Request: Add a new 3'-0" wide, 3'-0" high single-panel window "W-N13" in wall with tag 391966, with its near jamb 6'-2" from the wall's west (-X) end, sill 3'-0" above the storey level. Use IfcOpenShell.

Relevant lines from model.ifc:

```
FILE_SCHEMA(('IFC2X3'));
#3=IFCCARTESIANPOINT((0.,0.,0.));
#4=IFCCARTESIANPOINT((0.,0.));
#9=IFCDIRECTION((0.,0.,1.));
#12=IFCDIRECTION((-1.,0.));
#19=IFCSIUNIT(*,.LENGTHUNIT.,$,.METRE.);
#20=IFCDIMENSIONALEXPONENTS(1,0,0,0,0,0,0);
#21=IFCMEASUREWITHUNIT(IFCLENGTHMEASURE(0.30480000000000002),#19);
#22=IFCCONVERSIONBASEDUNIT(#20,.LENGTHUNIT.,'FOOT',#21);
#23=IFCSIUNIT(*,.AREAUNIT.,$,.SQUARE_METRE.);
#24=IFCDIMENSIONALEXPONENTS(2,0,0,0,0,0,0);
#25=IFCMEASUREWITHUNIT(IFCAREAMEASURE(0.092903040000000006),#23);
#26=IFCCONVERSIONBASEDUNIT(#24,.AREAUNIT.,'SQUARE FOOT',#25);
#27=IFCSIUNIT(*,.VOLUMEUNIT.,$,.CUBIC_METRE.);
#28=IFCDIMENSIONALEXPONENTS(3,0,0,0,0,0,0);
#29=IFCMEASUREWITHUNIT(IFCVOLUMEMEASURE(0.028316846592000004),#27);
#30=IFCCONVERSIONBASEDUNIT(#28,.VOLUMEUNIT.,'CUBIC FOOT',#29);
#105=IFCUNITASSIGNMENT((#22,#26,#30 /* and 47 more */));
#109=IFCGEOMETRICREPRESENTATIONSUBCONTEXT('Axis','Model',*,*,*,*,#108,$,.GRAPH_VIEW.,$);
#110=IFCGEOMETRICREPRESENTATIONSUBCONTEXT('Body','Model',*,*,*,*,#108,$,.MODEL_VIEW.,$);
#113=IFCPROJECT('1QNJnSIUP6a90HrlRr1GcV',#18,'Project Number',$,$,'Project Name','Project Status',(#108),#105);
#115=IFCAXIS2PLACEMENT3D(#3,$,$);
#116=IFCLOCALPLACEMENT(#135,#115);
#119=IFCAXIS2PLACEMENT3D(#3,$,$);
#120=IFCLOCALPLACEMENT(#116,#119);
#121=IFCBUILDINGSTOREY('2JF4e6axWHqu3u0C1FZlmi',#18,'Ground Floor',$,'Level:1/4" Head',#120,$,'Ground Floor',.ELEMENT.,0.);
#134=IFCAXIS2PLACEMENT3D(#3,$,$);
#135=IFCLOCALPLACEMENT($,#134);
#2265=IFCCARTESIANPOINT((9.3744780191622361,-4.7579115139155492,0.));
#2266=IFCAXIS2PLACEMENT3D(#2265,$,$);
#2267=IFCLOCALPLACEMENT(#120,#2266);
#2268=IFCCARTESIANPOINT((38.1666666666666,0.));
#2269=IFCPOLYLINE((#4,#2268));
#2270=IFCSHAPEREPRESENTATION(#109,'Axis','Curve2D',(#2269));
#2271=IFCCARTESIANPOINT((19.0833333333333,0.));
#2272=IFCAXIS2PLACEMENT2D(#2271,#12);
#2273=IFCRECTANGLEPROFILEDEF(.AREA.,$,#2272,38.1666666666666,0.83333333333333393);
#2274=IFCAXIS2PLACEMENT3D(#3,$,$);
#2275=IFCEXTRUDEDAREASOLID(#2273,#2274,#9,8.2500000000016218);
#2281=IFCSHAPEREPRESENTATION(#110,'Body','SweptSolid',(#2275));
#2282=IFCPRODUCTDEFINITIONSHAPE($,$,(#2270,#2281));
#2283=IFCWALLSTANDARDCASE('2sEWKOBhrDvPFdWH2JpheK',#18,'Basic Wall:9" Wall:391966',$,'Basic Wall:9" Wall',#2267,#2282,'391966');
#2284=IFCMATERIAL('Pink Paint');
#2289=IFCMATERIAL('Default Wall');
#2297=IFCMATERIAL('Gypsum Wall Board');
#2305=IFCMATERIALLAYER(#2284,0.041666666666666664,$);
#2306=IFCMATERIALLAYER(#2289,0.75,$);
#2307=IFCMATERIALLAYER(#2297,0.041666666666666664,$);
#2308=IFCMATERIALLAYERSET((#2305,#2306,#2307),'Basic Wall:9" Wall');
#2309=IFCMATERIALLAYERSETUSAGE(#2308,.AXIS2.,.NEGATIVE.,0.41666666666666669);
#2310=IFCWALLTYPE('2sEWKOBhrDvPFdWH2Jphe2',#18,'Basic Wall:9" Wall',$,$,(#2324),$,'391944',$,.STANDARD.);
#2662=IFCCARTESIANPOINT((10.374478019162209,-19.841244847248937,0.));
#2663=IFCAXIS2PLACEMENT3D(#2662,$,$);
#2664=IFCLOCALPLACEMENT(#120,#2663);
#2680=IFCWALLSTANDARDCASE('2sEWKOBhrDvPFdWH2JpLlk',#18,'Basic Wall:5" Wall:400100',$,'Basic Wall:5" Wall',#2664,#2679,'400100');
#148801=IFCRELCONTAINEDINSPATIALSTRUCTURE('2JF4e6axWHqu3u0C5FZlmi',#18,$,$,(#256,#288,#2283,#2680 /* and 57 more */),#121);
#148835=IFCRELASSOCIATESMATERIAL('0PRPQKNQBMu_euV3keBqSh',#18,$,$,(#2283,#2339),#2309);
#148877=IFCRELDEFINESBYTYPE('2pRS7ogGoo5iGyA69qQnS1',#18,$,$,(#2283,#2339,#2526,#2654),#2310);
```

```python
import numpy as np
import ifcopenshell
import ifcopenshell.api.feature
import ifcopenshell.api.geometry
import ifcopenshell.api.root
import ifcopenshell.api.spatial
import ifcopenshell.api.type
import ifcopenshell.geom
import ifcopenshell.util.element
import ifcopenshell.util.placement
import ifcopenshell.util.representation
import ifcopenshell.util.shape
import ifcopenshell.util.unit

model = ifcopenshell.open("model.ifc")
unit_scale = ifcopenshell.util.unit.calculate_unit_scale(model)
settings = ifcopenshell.geom.settings()


def volume(element):
    """Net volume in cubic metres, openings subtracted."""
    shape = ifcopenshell.geom.create_shape(settings, element)
    return ifcopenshell.util.shape.get_volume(shape.geometry)


wall = model.by_guid("2sEWKOBhrDvPFdWH2JpheK")
storey = ifcopenshell.util.element.get_container(wall, ifc_class="IfcBuildingStorey")
context = ifcopenshell.util.representation.get_context(model, "Model", "Body", "MODEL_VIEW")
before = volume(wall)

width, height, from_end, sill = 0.9144, 0.9144, 1.8796, 0.9144  # metres

# The wall runs along its own X axis, and the end named is its -X end.
wall_shape = ifcopenshell.geom.create_shape(settings, wall)
x, y, z = ifcopenshell.util.shape.get_vertices(wall_shape.geometry).T
start = x.min() + from_end
face, thickness = float(y.min()), float(y.max() - y.min())
wall_matrix = ifcopenshell.util.placement.get_local_placement(wall.ObjectPlacement)
level = ifcopenshell.util.placement.get_local_placement(storey.ObjectPlacement)[2, 3]


def in_wall(x, y):
    """Placement at x, y metres in the wall's axes, at sill height."""
    matrix = wall_matrix.copy()
    matrix[:, 3] = wall_matrix @ np.array([x / unit_scale, y / unit_scale, 0.0, 1.0])
    matrix[2, 3] = level + sill / unit_scale
    return matrix


# Opening: a box that overshoots both wall faces by 50 mm.
opening = ifcopenshell.api.root.create_entity(model, ifc_class="IfcOpeningElement")
box = ifcopenshell.api.geometry.add_wall_representation(
    model, context=context, length=width, height=height, thickness=thickness + 0.1
)
ifcopenshell.api.geometry.assign_representation(model, product=opening, representation=box)
ifcopenshell.api.geometry.edit_object_placement(model, product=opening, matrix=in_wall(start, face - 0.05), is_si=False)
ifcopenshell.api.feature.add_feature(model, feature=opening, element=wall)

window = ifcopenshell.api.root.create_entity(model, ifc_class="IfcWindow", name="W-N13")
window.OverallWidth, window.OverallHeight = width / unit_scale, height / unit_scale
body = ifcopenshell.api.geometry.add_window_representation(
    model,
    context=context,
    overall_width=window.OverallWidth,
    overall_height=window.OverallHeight,
    partition_type="SINGLE_PANEL",
)
ifcopenshell.api.geometry.assign_representation(model, product=window, representation=body)
ifcopenshell.api.spatial.assign_container(model, products=[window], relating_structure=storey)
fills = ifcopenshell.api.feature.add_filling(model, opening=opening, element=window)
fills.OwnerHistory = window.OwnerHistory  # required in IFC2X3

# IFC2X3 keeps the operation on the window style.
style = ifcopenshell.api.root.create_entity(model, ifc_class="IfcWindowStyle", name="W-N13")
style.OperationType, style.ConstructionType = "SINGLE_PANEL", "NOTDEFINED"
style.ParameterTakesPrecedence = style.Sizeable = False
ifcopenshell.api.type.assign_type(model, related_objects=[window], relating_type=style)

# Centre the window in the wall's thickness.
ifcopenshell.api.geometry.edit_object_placement(model, product=window, matrix=in_wall(start, face), is_si=False)
window_shape = ifcopenshell.geom.create_shape(settings, window)
depth = ifcopenshell.util.shape.get_vertices(window_shape.geometry)[:, 1]
offset = face + thickness / 2 - (depth.min() + depth.max()) / 2
ifcopenshell.api.geometry.edit_object_placement(model, product=window, matrix=in_wall(start, offset), is_si=False)

after = volume(wall)

print(f"wall volume {before:.3f} -> {after:.3f} m3")

model.write("model_updated.ifc")
```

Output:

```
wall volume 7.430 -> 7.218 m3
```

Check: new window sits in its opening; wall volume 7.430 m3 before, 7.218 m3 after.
